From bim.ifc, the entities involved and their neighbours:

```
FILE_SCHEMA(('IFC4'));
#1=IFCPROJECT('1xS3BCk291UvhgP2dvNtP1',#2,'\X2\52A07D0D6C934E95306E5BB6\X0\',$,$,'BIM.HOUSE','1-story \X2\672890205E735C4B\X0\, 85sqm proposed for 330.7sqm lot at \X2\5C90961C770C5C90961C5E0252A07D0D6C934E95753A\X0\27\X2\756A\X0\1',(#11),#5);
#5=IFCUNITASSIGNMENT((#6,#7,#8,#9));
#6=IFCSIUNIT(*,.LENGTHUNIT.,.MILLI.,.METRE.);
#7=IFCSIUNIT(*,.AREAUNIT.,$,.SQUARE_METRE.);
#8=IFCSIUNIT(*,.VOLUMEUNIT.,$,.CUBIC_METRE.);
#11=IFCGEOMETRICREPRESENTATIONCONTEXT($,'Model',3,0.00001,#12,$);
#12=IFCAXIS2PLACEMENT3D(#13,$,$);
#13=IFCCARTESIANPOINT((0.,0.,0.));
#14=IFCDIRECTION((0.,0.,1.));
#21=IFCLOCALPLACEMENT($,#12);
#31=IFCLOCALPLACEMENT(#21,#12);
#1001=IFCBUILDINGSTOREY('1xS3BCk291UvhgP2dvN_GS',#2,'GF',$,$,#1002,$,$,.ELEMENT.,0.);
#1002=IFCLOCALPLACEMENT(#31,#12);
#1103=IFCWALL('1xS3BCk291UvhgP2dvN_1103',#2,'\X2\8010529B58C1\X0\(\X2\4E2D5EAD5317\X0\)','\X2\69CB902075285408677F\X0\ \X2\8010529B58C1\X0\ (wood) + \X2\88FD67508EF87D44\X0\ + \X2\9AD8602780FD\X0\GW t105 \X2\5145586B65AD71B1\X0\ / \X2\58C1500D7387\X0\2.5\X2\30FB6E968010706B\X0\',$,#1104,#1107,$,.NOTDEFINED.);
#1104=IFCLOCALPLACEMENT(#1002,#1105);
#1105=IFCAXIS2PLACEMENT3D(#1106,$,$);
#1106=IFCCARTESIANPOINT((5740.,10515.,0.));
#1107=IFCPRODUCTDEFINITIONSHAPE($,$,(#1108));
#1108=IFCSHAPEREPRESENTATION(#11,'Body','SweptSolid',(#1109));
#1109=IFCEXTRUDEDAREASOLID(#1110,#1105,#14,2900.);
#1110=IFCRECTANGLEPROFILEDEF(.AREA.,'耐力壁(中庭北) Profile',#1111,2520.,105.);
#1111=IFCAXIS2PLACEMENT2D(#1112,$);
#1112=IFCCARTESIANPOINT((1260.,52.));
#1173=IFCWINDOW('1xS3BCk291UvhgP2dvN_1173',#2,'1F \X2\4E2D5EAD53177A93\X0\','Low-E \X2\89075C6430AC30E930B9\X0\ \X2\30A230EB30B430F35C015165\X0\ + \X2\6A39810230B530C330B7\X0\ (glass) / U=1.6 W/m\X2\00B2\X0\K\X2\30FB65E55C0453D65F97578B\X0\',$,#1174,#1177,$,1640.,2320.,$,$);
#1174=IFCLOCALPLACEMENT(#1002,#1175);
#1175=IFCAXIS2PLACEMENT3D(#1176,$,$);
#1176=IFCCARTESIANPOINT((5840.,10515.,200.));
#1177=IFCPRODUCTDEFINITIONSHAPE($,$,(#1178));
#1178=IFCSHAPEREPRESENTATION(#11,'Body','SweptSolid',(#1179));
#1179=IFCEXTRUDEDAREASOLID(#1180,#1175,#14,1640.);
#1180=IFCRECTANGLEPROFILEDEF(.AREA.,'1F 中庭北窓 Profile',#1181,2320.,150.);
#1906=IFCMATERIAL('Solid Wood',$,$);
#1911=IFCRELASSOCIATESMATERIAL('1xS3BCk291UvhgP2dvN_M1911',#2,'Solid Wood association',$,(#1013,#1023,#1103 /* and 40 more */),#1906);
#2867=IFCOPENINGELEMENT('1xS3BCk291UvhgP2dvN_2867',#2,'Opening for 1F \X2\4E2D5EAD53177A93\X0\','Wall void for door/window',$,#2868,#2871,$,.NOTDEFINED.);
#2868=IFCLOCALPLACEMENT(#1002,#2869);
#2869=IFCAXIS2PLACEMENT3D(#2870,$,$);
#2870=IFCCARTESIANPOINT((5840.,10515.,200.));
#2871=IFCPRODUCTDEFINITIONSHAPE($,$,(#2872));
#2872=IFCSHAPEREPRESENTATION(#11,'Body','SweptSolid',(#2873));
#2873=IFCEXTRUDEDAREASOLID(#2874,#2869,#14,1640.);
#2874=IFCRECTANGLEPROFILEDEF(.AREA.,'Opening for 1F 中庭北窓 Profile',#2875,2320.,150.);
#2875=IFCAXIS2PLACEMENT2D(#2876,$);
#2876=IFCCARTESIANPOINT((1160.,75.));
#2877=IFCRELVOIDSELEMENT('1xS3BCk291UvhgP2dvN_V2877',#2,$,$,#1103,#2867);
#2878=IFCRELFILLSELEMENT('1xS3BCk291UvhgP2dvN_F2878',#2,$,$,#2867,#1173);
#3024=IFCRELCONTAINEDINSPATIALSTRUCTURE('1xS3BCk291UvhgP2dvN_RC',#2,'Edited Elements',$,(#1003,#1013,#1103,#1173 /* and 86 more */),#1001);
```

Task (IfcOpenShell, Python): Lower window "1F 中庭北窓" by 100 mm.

```python
import numpy as np
import ifcopenshell
import ifcopenshell.api.geometry
import ifcopenshell.util.placement
import ifcopenshell.util.unit

model = ifcopenshell.open("bim.ifc")
unit_scale = ifcopenshell.util.unit.calculate_unit_scale(model)

window = model.by_id(1173)
opening = window.FillsVoids[0].RelatingOpeningElement
dz = -0.1 / unit_scale

shift = np.array([0.0, 0.0, dz])
# The window is not placed relative to its opening, so move both.
for product in (opening, window):
    matrix = ifcopenshell.util.placement.get_local_placement(product.ObjectPlacement)
    matrix[:3, 3] += shift
    ifcopenshell.api.geometry.edit_object_placement(model, product=product, matrix=matrix, is_si=False)

print(f"moved by {dz * unit_scale:+.3f} m")

model.write("bim_updated.ifc")
```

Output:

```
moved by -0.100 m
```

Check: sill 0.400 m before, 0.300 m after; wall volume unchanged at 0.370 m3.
